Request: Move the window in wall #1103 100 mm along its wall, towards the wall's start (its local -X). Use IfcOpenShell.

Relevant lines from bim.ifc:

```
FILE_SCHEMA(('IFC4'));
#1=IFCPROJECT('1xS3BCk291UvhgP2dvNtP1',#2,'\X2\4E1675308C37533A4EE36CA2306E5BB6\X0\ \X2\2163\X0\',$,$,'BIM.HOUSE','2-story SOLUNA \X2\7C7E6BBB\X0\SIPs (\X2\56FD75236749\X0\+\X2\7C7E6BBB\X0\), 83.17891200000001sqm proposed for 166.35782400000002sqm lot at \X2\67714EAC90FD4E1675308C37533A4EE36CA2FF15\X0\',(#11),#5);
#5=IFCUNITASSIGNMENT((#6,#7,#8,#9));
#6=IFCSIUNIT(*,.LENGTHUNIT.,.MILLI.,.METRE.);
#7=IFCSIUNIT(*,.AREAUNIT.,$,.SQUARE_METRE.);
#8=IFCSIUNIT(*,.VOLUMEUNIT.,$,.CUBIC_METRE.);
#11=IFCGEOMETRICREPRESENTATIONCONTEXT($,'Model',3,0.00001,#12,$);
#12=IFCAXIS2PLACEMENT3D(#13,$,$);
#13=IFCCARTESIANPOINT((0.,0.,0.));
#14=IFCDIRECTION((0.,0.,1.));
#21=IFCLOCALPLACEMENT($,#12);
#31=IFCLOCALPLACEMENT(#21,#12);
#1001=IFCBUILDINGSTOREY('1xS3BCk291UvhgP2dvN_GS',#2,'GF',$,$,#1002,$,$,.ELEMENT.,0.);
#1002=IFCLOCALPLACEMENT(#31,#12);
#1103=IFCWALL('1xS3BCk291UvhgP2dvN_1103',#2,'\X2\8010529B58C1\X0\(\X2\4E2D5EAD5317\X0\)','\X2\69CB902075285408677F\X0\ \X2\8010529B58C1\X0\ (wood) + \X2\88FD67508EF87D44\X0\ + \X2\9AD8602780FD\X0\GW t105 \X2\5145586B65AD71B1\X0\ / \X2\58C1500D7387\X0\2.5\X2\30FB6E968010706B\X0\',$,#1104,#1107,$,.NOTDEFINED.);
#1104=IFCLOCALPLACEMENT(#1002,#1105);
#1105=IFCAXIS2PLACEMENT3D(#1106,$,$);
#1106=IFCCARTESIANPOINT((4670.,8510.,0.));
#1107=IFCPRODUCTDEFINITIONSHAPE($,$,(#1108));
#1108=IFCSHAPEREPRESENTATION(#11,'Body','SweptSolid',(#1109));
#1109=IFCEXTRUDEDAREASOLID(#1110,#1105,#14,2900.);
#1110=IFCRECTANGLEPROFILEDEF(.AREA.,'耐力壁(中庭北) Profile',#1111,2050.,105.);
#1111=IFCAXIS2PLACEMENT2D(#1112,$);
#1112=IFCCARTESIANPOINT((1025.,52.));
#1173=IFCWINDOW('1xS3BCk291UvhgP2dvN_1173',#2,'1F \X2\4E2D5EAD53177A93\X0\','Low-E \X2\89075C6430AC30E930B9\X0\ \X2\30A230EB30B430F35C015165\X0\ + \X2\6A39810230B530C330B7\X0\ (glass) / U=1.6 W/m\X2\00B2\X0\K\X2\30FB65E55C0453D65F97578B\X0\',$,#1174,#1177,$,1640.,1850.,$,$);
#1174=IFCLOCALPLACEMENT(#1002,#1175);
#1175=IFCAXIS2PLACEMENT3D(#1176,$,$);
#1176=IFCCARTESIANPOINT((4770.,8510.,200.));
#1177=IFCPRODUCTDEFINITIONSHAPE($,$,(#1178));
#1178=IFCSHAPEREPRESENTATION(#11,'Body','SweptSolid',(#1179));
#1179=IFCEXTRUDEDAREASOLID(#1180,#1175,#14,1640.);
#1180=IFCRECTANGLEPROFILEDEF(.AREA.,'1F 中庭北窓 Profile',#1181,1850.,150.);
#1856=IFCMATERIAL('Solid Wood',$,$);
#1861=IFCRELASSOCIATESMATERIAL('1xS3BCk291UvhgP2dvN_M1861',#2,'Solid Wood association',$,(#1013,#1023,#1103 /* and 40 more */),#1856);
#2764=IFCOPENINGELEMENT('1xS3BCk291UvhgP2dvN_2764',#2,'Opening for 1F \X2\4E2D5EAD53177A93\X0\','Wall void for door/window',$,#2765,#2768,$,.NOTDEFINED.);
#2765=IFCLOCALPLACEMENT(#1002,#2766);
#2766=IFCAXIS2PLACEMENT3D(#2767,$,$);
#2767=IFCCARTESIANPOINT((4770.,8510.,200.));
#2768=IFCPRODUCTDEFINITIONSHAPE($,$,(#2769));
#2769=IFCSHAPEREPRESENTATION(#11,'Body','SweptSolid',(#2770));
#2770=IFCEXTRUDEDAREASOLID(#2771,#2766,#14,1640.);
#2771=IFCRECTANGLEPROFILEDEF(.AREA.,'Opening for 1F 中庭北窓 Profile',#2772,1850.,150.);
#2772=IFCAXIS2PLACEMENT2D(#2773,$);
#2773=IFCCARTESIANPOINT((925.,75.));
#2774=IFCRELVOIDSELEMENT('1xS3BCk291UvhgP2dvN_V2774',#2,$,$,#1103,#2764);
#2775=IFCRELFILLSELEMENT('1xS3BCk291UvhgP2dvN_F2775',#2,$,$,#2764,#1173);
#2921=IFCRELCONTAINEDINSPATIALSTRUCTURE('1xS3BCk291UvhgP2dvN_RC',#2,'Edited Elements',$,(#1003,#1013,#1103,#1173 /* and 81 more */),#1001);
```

```python
import ifcopenshell
import ifcopenshell.api.geometry
import ifcopenshell.util.placement
import ifcopenshell.util.unit

model = ifcopenshell.open("bim.ifc")
unit_scale = ifcopenshell.util.unit.calculate_unit_scale(model)

window = model.by_id(1173)
opening = window.FillsVoids[0].RelatingOpeningElement
wall = opening.VoidsElements[0].RelatingBuildingElement

wall_matrix = ifcopenshell.util.placement.get_local_placement(wall.ObjectPlacement)
shift = wall_matrix[:3, 0] * -0.1 / unit_scale
before = ifcopenshell.util.placement.get_local_placement(window.ObjectPlacement)[:3, 3].copy()

# The window is not placed relative to its opening, so move both.
for product in (opening, window):
    matrix = ifcopenshell.util.placement.get_local_placement(product.ObjectPlacement)
    matrix[:3, 3] += shift
    ifcopenshell.api.geometry.edit_object_placement(model, product=product, matrix=matrix, is_si=False)

after = ifcopenshell.util.placement.get_local_placement(window.ObjectPlacement)[:3, 3]
print("window moved by", (after - before).round(3) + 0.0)

model.write("bim_edited.ifc")
```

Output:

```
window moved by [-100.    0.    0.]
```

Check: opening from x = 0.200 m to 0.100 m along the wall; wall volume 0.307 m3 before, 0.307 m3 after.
